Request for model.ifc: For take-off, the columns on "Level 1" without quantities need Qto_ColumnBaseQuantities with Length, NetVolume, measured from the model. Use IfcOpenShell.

First a look at what the model holds.

```python
import ifcopenshell
import ifcopenshell.util.element
import ifcopenshell.util.unit

model = ifcopenshell.open("model.ifc")
print(model.schema)
for unit_type in ("LENGTHUNIT", "AREAUNIT", "VOLUMEUNIT"):
    print(unit_type, ifcopenshell.util.unit.calculate_unit_scale(model, unit_type))
storey = next(s for s in model.by_type("IfcBuildingStorey") if s.Name == "Level 1")
columns = [e for e in ifcopenshell.util.element.get_decomposition(storey) if e.is_a("IfcColumn")]
for e in sorted(columns, key=lambda e: e.id()):
    print(e.id(), e.is_a(), e.Name, list(ifcopenshell.util.element.get_psets(e, qtos_only=True)), sep=" | ")
```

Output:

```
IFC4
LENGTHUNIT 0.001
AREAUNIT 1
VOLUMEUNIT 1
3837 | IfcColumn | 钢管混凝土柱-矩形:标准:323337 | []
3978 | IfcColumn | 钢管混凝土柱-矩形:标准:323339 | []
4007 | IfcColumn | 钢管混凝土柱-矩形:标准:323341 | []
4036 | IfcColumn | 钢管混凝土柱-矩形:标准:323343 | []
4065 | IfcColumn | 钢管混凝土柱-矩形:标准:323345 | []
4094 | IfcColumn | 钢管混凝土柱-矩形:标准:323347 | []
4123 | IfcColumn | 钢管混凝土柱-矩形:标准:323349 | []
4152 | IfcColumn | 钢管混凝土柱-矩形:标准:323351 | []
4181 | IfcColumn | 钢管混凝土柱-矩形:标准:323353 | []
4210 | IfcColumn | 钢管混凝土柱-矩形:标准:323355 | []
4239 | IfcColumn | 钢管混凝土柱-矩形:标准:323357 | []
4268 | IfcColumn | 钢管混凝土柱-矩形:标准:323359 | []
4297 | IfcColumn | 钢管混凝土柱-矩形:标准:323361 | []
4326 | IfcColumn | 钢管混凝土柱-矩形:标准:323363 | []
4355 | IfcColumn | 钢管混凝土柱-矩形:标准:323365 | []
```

```python
import ifcopenshell
import ifcopenshell.api.pset
import ifcopenshell.geom
import ifcopenshell.util.element
import ifcopenshell.util.shape
import ifcopenshell.util.unit

model = ifcopenshell.open("model.ifc")
unit_scale = ifcopenshell.util.unit.calculate_unit_scale(model)
volume_scale = ifcopenshell.util.unit.calculate_unit_scale(model, "VOLUMEUNIT")
settings = ifcopenshell.geom.settings()

storey = next(s for s in model.by_type("IfcBuildingStorey") if s.Name == "Level 1")
columns = [e for e in ifcopenshell.util.element.get_decomposition(storey) if e.is_a("IfcColumn")]

for e in sorted(columns, key=lambda e: e.id()):
    if ifcopenshell.util.element.get_psets(e, qtos_only=True, should_inherit=False):
        continue
    # Geometry comes back in metres, in the element's own axes.
    shape = ifcopenshell.geom.create_shape(settings, e)
    values = {
        "Length": ifcopenshell.util.shape.get_z(shape.geometry) / unit_scale,
        "NetVolume": ifcopenshell.util.shape.get_volume(shape.geometry) / volume_scale,
    }
    qto = ifcopenshell.api.pset.add_qto(model, product=e, name="Qto_ColumnBaseQuantities")
    ifcopenshell.api.pset.edit_qto(model, qto=qto, properties=values)
    print(e.id(), {k: round(v, 3) for k, v in values.items()})

model.write("model-out.ifc")
```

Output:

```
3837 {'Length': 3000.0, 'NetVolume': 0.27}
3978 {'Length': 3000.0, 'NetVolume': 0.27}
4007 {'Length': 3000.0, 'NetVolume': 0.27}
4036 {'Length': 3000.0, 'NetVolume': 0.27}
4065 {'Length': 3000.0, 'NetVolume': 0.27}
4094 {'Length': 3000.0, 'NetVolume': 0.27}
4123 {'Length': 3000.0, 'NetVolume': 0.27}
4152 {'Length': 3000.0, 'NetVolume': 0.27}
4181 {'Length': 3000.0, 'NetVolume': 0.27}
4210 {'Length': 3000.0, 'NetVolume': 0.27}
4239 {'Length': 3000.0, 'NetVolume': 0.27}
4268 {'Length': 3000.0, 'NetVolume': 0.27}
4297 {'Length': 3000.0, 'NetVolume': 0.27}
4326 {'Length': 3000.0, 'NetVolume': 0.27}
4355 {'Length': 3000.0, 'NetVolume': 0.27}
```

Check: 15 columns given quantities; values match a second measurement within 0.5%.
